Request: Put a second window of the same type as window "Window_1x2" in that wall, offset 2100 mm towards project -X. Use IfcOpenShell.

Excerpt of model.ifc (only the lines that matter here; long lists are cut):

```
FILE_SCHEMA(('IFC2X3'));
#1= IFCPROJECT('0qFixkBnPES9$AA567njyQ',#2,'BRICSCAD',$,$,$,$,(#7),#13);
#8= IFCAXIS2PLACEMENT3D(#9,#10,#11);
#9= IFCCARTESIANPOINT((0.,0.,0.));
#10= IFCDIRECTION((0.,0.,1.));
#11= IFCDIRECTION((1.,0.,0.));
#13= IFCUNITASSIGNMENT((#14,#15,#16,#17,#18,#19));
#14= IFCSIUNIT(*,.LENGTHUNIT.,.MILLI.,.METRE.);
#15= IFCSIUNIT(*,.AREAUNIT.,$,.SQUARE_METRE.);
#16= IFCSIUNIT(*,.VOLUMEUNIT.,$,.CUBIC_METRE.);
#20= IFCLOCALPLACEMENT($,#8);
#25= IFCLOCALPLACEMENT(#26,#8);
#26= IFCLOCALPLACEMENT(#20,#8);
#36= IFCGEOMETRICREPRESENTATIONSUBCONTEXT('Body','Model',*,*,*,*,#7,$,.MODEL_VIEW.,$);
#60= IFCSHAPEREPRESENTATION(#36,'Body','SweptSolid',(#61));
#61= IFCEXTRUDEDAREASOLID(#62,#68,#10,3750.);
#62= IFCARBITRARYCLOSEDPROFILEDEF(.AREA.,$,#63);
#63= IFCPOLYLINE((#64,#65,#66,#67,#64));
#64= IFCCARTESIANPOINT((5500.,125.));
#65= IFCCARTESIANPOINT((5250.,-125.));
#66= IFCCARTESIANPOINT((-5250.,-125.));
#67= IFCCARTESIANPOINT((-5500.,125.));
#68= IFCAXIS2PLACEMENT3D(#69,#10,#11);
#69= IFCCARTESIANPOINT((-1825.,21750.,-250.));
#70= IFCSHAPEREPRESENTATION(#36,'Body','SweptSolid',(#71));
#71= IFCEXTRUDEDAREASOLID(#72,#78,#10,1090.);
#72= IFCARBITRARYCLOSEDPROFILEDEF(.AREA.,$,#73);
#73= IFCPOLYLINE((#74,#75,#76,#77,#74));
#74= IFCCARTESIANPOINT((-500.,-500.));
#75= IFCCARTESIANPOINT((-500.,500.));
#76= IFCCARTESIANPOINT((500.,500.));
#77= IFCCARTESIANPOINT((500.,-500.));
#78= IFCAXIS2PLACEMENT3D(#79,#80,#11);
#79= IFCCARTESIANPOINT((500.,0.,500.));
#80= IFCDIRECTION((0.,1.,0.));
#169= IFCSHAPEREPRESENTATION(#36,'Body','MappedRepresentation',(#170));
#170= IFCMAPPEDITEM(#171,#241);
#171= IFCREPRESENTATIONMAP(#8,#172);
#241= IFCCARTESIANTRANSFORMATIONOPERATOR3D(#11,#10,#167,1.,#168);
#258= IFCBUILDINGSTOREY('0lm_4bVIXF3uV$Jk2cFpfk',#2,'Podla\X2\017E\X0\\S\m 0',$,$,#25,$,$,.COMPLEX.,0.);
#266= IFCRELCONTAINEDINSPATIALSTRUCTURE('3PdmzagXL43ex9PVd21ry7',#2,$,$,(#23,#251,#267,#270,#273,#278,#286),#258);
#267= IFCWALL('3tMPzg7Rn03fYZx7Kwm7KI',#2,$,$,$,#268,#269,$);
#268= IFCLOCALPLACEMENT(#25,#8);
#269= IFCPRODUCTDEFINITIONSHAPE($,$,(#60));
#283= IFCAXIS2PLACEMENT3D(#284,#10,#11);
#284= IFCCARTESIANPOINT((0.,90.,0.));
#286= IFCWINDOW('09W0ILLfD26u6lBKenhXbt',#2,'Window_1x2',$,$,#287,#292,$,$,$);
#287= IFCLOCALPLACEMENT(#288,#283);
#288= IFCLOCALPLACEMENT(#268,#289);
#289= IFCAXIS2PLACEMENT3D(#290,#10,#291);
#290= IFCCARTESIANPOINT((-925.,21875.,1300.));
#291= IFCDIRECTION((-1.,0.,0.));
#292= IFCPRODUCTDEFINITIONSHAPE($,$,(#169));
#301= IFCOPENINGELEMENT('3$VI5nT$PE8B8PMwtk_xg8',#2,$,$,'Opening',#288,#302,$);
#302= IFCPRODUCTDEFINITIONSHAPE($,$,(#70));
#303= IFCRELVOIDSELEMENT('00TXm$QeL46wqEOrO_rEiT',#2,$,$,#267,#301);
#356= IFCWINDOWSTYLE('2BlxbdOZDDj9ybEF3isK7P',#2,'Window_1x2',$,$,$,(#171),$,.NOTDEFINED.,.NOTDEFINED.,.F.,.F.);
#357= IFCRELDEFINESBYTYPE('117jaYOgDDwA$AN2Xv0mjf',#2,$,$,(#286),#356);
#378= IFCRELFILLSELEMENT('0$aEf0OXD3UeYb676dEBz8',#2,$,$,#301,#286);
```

```python
import ifcopenshell
import ifcopenshell.api.feature
import ifcopenshell.api.geometry
import ifcopenshell.api.root
import ifcopenshell.geom
import ifcopenshell.util.element
import ifcopenshell.util.placement
import ifcopenshell.util.shape

model = ifcopenshell.open("model.ifc")
settings = ifcopenshell.geom.settings()


def volume(element):
    """Net volume in cubic metres, openings subtracted."""
    shape = ifcopenshell.geom.create_shape(settings, element)
    return ifcopenshell.util.shape.get_volume(shape.geometry)


def reuse_history(source, copy):
    """copy_class also copies each property set's owner history, people and application; keep the originals."""
    for rel in copy.IsDefinedBy:
        if rel.is_a("IfcRelDefinesByProperties") and (history := rel.RelatingPropertyDefinition.OwnerHistory):
            rel.RelatingPropertyDefinition.OwnerHistory = source.OwnerHistory
            ifcopenshell.util.element.remove_deep2(model, history)


window = model.by_guid("09W0ILLfD26u6lBKenhXbt")
opening = window.FillsVoids[0].RelatingOpeningElement
wall = opening.VoidsElements[0].RelatingBuildingElement
before = volume(wall)
shift = ifcopenshell.util.placement.get_local_placement(wall.ObjectPlacement)[:3, 0] * -2100.0

# copy_class copies the void relationship, type, container and properties, but no geometry.
new_opening = ifcopenshell.api.root.copy_class(model, product=opening)
new_opening.Representation = ifcopenshell.util.element.copy_deep(
    model, opening.Representation, exclude=["IfcGeometricRepresentationContext", "IfcRepresentationMap"]
)
new_window = ifcopenshell.api.root.copy_class(model, product=window)
new_window.Representation = ifcopenshell.util.element.copy_deep(
    model, window.Representation, exclude=["IfcGeometricRepresentationContext", "IfcRepresentationMap"]
)
reuse_history(window, new_window)
fills = ifcopenshell.api.feature.add_filling(model, opening=new_opening, element=new_window)
fills.OwnerHistory = new_window.OwnerHistory  # required in IFC2X3

for old, new in ((opening, new_opening), (window, new_window)):
    matrix = ifcopenshell.util.placement.get_local_placement(old.ObjectPlacement)
    matrix[:3, 3] += shift
    ifcopenshell.api.geometry.edit_object_placement(model, product=new, matrix=matrix, is_si=False)

after = volume(wall)

print(f"wall volume {before:.3f} -> {after:.3f} m3")

model.write("model_edited.ifc")
```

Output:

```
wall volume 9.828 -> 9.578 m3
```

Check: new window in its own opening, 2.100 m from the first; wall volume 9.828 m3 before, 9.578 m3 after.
